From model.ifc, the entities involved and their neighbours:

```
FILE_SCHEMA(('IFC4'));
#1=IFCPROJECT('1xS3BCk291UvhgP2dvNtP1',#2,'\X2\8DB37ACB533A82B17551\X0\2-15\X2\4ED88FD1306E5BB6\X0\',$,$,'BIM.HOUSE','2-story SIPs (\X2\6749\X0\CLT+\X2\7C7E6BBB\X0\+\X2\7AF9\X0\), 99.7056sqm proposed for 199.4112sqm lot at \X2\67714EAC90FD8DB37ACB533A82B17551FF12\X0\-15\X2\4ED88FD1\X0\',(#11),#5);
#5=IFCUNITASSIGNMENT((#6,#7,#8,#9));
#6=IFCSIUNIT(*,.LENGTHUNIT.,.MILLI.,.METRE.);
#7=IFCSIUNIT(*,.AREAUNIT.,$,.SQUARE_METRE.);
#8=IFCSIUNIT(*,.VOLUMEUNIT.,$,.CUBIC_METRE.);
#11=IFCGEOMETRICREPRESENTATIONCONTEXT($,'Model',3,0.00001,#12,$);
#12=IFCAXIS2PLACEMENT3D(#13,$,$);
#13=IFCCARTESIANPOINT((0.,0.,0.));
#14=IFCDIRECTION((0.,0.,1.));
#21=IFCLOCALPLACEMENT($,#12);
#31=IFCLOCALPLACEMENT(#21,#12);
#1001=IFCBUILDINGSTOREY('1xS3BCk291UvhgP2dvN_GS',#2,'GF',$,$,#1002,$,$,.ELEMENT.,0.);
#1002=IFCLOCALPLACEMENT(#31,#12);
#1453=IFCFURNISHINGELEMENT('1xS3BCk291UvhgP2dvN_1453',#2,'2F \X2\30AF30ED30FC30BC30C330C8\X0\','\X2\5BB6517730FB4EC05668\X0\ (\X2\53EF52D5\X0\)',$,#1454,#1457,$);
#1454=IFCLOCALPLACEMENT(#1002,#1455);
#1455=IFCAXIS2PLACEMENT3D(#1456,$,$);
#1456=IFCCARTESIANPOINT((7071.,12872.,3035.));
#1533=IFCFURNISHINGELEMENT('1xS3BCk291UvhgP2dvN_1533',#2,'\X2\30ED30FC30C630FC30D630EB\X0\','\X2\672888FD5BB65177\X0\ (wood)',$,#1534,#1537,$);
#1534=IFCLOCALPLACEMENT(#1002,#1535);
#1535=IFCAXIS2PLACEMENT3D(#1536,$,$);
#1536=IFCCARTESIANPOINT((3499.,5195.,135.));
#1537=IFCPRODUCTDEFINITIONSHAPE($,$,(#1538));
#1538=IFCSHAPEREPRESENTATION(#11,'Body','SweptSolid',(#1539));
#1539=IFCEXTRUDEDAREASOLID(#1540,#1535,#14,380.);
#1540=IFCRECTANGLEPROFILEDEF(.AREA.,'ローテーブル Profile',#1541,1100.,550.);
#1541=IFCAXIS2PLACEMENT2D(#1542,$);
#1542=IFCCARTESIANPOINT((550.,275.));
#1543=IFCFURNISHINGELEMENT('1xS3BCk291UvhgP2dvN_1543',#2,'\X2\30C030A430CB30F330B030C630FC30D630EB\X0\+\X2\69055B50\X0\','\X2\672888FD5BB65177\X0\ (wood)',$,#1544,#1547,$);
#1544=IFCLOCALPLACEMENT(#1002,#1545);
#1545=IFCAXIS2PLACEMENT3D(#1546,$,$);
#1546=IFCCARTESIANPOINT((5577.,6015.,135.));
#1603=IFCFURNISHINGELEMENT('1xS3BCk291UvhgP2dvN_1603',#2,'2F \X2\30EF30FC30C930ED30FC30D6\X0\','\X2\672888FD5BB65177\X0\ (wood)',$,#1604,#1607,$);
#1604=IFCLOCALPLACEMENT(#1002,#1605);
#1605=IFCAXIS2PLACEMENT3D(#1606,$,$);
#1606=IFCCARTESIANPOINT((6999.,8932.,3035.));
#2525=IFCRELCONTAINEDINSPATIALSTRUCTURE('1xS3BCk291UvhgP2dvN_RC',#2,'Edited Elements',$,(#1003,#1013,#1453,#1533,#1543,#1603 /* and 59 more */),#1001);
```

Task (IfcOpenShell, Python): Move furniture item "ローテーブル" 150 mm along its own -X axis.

```python
import ifcopenshell
import ifcopenshell.api.geometry
import ifcopenshell.util.placement
import ifcopenshell.util.unit

model = ifcopenshell.open("model.ifc")
unit_scale = ifcopenshell.util.unit.calculate_unit_scale(model)

item = model.by_guid("1xS3BCk291UvhgP2dvN_1533")
matrix = ifcopenshell.util.placement.get_local_placement(item.ObjectPlacement)
matrix[:3, 3] -= matrix[:3, 0] * 0.15 / unit_scale
ifcopenshell.api.geometry.edit_object_placement(model, product=item, matrix=matrix, is_si=False)

print(ifcopenshell.util.placement.get_local_placement(item.ObjectPlacement).round(3) + 0.0)

model.write("model_updated.ifc")
```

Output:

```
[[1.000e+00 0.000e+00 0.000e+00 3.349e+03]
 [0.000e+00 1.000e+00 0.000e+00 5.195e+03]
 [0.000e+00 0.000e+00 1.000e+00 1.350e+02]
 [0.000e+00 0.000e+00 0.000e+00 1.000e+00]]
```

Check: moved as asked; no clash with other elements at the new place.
